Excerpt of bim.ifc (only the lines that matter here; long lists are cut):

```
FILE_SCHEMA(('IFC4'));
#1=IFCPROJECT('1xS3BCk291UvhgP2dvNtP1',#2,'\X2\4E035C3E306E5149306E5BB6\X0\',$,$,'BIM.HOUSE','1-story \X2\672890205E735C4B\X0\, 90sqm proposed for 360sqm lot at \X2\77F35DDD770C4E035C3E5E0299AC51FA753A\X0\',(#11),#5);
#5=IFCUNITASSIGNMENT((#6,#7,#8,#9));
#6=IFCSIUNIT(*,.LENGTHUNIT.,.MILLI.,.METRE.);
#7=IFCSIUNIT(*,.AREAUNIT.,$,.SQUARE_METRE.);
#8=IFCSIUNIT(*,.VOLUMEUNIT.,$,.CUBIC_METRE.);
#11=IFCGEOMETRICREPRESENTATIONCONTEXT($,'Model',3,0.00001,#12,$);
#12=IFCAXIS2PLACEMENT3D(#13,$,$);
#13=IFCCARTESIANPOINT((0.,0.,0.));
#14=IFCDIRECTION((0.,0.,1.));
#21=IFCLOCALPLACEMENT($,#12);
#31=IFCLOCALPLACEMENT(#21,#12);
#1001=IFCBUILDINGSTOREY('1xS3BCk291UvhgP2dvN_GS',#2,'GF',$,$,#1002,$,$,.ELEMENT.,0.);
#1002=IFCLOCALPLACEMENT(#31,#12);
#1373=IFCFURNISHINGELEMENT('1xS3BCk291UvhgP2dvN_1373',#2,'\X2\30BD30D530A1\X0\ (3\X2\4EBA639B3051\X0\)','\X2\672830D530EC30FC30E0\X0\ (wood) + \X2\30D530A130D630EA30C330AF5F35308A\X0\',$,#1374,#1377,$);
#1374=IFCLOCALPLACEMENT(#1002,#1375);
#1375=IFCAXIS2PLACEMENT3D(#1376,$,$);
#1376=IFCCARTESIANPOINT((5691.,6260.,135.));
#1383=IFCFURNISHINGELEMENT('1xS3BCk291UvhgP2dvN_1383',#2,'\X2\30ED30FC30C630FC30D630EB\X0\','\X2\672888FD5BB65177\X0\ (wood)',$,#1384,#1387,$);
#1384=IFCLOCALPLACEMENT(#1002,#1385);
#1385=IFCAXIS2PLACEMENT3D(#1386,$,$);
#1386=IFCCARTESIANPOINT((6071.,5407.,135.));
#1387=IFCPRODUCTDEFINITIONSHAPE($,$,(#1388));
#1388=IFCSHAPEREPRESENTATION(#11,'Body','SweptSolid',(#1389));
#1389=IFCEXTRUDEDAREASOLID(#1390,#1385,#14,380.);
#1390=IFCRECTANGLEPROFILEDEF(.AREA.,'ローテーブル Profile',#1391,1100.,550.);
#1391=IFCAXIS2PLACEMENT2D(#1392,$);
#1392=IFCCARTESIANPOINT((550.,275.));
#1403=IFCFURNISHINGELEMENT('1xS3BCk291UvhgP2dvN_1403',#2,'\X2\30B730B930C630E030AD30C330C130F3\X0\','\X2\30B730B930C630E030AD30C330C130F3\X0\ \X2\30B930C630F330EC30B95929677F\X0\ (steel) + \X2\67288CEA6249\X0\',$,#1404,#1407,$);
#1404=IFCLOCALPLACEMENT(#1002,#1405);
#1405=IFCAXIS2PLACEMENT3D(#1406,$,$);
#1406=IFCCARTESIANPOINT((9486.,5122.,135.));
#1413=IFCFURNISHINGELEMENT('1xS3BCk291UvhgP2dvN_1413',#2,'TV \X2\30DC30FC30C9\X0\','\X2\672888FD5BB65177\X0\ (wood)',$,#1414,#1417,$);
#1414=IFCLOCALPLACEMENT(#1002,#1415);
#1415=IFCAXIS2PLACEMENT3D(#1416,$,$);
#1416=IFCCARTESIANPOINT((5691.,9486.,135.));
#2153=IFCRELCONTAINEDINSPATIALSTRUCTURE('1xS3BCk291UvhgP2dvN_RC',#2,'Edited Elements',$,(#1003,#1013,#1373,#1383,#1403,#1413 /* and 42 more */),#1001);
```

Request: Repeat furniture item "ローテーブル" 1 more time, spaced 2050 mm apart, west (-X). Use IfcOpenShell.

```python
import numpy as np
import ifcopenshell
import ifcopenshell.api.geometry
import ifcopenshell.api.root
import ifcopenshell.util.element
import ifcopenshell.util.placement

model = ifcopenshell.open("bim.ifc")


def reuse_history(source, copy):
    """copy_class also copies each property set's owner history, people and application; keep the originals."""
    for rel in copy.IsDefinedBy:
        if rel.is_a("IfcRelDefinesByProperties") and (history := rel.RelatingPropertyDefinition.OwnerHistory):
            rel.RelatingPropertyDefinition.OwnerHistory = source.OwnerHistory
            ifcopenshell.util.element.remove_deep2(model, history)


source = model.by_guid("1xS3BCk291UvhgP2dvN_1383")
base = ifcopenshell.util.placement.get_local_placement(source.ObjectPlacement)
step = np.array([-1.0, 0.0, 0.0]) * 2050.0

for i in range(1, 2):
    copy = ifcopenshell.api.root.copy_class(model, product=source)
    copy.Representation = ifcopenshell.util.element.copy_deep(
        model, source.Representation, exclude=["IfcGeometricRepresentationContext", "IfcRepresentationMap"]
    )
    reuse_history(source, copy)
    matrix = base.copy()
    matrix[:3, 3] += i * step
    print("added at", matrix[:3, 3].round(3) + 0.0)
    ifcopenshell.api.geometry.edit_object_placement(model, product=copy, matrix=matrix, is_si=False)

model.write("bim-out.ifc")
```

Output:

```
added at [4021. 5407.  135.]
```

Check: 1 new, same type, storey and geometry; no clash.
